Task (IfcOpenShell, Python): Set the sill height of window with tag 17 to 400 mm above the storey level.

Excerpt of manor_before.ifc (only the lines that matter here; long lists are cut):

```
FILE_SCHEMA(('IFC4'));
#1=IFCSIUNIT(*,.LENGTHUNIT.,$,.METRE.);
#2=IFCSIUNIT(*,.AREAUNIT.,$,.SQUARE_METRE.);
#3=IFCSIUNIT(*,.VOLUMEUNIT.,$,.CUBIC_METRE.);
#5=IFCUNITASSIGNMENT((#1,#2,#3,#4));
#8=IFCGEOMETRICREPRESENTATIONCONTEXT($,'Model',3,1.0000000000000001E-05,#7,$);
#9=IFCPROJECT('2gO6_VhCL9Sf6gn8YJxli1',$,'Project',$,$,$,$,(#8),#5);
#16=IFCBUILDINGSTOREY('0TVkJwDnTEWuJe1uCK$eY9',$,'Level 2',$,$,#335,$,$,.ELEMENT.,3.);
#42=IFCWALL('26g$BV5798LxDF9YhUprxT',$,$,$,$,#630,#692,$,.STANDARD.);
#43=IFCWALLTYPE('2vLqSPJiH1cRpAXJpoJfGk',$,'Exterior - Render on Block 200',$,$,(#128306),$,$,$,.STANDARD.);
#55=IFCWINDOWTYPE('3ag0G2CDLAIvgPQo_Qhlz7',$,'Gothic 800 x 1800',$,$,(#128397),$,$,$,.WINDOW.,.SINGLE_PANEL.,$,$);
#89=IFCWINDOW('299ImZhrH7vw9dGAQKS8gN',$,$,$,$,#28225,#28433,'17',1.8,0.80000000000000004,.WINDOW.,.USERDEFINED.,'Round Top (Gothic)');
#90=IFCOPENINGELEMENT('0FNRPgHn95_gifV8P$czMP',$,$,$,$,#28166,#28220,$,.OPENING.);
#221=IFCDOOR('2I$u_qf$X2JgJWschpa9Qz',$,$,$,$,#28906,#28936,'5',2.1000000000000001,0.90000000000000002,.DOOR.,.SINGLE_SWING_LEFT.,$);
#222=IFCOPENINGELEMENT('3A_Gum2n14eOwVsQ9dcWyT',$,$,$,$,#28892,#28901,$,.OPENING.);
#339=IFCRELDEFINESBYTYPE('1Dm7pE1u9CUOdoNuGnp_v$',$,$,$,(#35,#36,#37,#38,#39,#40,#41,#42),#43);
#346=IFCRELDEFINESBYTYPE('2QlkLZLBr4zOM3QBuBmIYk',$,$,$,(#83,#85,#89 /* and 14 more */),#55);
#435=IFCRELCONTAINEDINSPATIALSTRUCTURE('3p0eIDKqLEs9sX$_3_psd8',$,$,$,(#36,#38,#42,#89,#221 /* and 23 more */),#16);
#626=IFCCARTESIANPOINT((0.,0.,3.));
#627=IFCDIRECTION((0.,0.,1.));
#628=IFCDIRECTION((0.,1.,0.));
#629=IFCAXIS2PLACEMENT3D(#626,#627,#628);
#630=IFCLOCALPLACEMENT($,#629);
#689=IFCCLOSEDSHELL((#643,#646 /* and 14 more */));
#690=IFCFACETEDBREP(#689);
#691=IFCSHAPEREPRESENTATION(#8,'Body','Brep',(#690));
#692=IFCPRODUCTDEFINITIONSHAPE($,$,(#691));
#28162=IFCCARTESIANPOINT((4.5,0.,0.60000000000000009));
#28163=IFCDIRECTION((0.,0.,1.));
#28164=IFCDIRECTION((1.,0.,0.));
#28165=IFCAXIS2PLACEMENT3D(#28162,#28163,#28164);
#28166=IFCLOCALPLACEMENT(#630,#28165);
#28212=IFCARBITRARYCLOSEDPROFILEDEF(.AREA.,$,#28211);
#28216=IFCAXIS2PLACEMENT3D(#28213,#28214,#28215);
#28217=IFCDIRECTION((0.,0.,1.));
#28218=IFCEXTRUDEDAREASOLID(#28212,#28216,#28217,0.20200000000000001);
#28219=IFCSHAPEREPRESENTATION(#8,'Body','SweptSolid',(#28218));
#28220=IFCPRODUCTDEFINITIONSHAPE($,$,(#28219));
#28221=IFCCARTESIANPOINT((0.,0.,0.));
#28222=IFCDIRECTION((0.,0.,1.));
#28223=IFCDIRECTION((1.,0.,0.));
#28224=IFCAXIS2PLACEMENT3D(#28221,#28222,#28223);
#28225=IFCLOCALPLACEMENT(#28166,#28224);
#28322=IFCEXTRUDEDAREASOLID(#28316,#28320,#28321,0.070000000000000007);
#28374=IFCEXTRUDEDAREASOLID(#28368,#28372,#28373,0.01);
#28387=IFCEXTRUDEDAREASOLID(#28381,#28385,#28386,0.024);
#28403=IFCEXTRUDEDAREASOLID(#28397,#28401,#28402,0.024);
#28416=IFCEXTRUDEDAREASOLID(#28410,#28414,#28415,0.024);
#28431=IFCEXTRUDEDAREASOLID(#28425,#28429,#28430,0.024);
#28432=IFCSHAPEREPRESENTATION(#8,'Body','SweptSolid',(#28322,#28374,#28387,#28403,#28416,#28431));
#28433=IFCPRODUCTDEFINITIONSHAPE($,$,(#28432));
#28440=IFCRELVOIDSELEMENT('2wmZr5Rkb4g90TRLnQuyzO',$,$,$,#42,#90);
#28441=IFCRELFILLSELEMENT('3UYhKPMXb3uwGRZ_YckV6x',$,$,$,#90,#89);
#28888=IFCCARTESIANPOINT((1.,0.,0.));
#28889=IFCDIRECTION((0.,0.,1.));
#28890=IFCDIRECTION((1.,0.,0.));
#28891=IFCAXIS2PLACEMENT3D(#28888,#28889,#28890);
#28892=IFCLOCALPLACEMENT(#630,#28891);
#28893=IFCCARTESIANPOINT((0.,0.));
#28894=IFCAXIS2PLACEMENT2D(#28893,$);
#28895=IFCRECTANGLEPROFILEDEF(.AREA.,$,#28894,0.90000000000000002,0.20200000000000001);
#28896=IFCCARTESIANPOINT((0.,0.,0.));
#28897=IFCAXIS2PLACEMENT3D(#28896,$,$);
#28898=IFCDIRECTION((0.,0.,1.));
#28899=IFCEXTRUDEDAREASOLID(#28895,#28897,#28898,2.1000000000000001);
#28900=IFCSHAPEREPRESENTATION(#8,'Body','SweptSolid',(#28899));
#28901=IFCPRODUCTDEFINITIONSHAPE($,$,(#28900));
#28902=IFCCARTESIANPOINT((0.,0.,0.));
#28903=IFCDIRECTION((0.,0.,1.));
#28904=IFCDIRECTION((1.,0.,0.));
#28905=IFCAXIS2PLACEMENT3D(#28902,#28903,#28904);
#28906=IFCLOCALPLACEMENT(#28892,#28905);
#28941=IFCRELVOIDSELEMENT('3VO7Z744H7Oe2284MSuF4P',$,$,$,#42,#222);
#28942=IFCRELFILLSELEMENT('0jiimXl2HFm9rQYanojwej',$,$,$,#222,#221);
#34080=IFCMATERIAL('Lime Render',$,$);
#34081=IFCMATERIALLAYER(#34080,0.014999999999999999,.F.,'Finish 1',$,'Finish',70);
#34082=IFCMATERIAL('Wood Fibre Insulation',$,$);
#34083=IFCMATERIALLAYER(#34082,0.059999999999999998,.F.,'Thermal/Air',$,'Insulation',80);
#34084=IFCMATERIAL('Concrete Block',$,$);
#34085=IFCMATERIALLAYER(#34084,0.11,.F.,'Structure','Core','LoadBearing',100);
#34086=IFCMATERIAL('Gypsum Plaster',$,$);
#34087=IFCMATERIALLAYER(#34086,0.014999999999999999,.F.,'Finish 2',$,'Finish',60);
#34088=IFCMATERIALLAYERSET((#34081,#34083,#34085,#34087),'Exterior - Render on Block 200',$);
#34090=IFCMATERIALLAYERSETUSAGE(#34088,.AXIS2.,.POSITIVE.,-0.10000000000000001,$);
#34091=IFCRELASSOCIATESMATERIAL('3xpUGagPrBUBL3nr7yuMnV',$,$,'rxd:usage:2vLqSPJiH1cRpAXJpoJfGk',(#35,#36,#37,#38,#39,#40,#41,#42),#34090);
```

```python
import numpy as np
import ifcopenshell
import ifcopenshell.api.geometry
import ifcopenshell.geom
import ifcopenshell.util.element
import ifcopenshell.util.placement
import ifcopenshell.util.shape
import ifcopenshell.util.unit

model = ifcopenshell.open("manor_before.ifc")
unit_scale = ifcopenshell.util.unit.calculate_unit_scale(model)

window = model.by_guid("299ImZhrH7vw9dGAQKS8gN")
opening = window.FillsVoids[0].RelatingOpeningElement
storey = ifcopenshell.util.element.get_container(window, ifc_class="IfcBuildingStorey")
level = ifcopenshell.util.placement.get_local_placement(storey.ObjectPlacement)[2, 3]

# The opening's origin need not be at the sill, so measure its lowest point.
shape = ifcopenshell.geom.create_shape(ifcopenshell.geom.settings(), opening)
bottom = ifcopenshell.util.shape.get_shape_bottom_elevation(shape, shape.geometry) / unit_scale
dz = level + 0.4 - bottom

shift = np.array([0.0, 0.0, dz])
# The window is placed relative to its opening, so it follows when the opening moves.
matrix = ifcopenshell.util.placement.get_local_placement(opening.ObjectPlacement)
matrix[:3, 3] += shift
ifcopenshell.api.geometry.edit_object_placement(
    model, product=opening, matrix=matrix, is_si=False, should_transform_children=True
)

print(f"moved by {dz * unit_scale:+.3f} m")

model.write("manor_before_updated.ifc")
```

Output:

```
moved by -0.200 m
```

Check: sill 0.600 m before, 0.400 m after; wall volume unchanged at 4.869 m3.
